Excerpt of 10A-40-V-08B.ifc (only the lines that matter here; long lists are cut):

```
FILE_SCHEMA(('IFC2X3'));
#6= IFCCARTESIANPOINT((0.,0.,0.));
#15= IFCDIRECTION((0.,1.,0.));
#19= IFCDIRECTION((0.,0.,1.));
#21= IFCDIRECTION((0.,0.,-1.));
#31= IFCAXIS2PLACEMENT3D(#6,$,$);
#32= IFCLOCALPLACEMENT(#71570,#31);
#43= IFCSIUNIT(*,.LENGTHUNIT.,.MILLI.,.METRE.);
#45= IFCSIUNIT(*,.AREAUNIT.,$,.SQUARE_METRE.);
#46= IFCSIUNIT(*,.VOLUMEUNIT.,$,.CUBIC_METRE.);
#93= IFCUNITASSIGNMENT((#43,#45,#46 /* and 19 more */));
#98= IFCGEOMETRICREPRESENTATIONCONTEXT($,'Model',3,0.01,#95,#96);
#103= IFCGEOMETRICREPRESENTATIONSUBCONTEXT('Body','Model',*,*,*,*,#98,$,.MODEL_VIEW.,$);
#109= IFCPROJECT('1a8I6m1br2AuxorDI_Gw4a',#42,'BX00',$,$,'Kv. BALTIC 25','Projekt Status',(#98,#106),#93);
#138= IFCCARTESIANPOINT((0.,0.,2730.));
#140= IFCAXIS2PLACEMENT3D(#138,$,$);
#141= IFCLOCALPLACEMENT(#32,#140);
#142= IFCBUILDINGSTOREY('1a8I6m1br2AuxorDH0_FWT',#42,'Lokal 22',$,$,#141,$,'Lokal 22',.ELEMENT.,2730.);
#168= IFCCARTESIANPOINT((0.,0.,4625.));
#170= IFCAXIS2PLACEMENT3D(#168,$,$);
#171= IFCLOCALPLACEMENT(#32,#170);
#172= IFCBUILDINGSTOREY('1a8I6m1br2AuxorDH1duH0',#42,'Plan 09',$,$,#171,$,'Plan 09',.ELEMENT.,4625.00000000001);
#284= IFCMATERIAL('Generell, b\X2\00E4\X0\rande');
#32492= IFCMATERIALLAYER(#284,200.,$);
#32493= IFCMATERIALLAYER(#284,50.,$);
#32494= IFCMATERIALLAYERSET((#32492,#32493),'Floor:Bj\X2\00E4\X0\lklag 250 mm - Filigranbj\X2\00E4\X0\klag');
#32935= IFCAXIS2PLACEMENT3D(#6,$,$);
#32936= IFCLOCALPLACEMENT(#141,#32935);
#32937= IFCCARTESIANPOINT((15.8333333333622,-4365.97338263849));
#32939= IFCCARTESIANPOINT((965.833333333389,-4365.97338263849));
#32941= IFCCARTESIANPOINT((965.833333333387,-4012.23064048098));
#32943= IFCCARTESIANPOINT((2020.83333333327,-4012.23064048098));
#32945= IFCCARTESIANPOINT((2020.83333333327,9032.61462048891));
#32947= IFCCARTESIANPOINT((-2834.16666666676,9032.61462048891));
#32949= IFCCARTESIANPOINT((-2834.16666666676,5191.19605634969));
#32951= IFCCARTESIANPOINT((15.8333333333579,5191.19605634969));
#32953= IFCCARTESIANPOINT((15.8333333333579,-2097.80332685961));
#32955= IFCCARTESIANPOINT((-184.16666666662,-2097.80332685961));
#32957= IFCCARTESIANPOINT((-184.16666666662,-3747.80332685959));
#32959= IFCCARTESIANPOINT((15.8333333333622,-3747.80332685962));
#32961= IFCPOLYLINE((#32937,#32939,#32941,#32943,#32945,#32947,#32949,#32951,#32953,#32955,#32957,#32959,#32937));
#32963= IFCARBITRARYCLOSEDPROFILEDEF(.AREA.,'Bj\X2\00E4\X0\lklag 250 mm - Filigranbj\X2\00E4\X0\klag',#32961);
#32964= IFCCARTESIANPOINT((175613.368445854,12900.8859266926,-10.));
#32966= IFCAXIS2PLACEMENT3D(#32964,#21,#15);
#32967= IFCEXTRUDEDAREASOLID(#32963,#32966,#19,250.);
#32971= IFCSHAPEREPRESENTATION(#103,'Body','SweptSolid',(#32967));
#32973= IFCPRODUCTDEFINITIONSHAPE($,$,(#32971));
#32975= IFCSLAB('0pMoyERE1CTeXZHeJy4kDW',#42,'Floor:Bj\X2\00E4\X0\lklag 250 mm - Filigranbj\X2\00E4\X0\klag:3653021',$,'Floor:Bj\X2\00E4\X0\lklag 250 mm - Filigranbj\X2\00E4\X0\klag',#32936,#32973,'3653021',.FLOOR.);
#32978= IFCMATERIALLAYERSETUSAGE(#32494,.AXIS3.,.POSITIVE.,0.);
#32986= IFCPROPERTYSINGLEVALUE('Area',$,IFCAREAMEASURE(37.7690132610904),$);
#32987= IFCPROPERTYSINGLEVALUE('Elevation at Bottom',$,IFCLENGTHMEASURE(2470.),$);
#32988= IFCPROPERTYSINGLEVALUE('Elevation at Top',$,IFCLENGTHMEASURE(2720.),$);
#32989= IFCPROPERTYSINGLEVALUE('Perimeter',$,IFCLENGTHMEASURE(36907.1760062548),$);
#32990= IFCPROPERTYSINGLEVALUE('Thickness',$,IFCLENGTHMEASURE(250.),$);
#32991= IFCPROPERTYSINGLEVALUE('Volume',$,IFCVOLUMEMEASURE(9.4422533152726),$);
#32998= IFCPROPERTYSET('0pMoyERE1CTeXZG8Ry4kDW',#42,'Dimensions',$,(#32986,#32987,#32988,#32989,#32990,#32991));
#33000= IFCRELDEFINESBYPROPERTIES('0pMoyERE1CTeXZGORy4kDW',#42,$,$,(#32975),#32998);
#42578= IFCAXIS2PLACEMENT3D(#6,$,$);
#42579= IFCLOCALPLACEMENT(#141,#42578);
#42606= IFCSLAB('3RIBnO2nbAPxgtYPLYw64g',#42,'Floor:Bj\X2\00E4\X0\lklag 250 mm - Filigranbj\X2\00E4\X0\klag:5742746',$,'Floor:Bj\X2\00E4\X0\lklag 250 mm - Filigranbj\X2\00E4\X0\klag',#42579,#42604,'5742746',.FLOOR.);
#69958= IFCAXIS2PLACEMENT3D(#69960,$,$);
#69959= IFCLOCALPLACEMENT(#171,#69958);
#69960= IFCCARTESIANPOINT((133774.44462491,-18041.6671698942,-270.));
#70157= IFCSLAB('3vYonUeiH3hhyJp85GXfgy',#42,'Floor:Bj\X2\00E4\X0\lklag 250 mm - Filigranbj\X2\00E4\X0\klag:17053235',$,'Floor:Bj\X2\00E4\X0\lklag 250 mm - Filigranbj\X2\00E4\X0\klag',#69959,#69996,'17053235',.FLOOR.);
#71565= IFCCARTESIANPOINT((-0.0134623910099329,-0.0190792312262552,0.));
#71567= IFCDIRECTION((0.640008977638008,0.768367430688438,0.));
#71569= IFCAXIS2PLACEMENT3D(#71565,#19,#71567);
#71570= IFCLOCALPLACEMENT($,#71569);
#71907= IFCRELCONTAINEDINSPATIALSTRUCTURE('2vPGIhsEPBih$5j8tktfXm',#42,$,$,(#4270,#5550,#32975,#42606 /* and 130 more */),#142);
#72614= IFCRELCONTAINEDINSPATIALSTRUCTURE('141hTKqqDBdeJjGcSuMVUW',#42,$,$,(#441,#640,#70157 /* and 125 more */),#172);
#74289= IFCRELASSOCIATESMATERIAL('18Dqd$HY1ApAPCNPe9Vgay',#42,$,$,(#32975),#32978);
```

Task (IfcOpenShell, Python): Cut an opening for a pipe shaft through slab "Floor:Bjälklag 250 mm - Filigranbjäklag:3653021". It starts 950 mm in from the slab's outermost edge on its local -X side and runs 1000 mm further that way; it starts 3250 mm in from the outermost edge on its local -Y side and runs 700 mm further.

```python
import numpy as np
import ifcopenshell
import ifcopenshell.api.feature
import ifcopenshell.api.geometry
import ifcopenshell.api.pset
import ifcopenshell.api.root
import ifcopenshell.geom
import ifcopenshell.util.element
import ifcopenshell.util.placement
import ifcopenshell.util.representation
import ifcopenshell.util.shape
import ifcopenshell.util.unit

model = ifcopenshell.open("10A-40-V-08B.ifc")
unit_scale = ifcopenshell.util.unit.calculate_unit_scale(model)
area_scale = ifcopenshell.util.unit.calculate_unit_scale(model, "AREAUNIT")
volume_scale = ifcopenshell.util.unit.calculate_unit_scale(model, "VOLUMEUNIT")
settings = ifcopenshell.geom.settings()


def volume(element):
    """Net volume in cubic metres, openings subtracted."""
    shape = ifcopenshell.geom.create_shape(settings, element)
    return ifcopenshell.util.shape.get_volume(shape.geometry)


slab = model.by_guid("0pMoyERE1CTeXZHeJy4kDW")
before = volume(slab)

# Extent in the slab's own axes, in metres. The edges named are its -X and -Y sides.
slab_shape = ifcopenshell.geom.create_shape(settings, slab)
vertices = ifcopenshell.util.shape.get_vertices(slab_shape.geometry)
x_min, y_min, bottom = vertices.min(axis=0)
top = vertices[:, 2].max()

opening = ifcopenshell.api.root.create_entity(model, ifc_class="IfcOpeningElement", name="Pipe shaft opening")
context = ifcopenshell.util.representation.get_context(model, "Model", "Body", "MODEL_VIEW")
width, depth = 1, 0.7
outline = [(0.0, 0.0), (width, 0.0), (width, depth), (0.0, depth), (0.0, 0.0)]
# Overshoot both faces by 50 mm so the cut is clean.
shape = ifcopenshell.api.geometry.add_slab_representation(
    model, context=context, depth=top - bottom + 0.1, polyline=outline
)
ifcopenshell.api.geometry.assign_representation(model, product=opening, representation=shape)

matrix = ifcopenshell.util.placement.get_local_placement(slab.ObjectPlacement)
matrix[:, 3] = matrix @ np.append(np.array([x_min + 0.95, y_min + 3.25, bottom - 0.05]) / unit_scale, 1.0)
ifcopenshell.api.geometry.edit_object_placement(model, product=opening, matrix=matrix, is_si=False)
ifcopenshell.api.feature.add_feature(model, feature=opening, element=slab)

after = volume(slab)

# Update the slab's stored quantities.
pset = model.by_id(ifcopenshell.util.element.get_pset(slab, "Dimensions", should_inherit=False)["id"])
ifcopenshell.api.pset.edit_pset(model, pset=pset, properties={
    "Area": model.create_entity("IfcAreaMeasure", after / (top - bottom) / area_scale),
    "Volume": model.create_entity("IfcVolumeMeasure", after / volume_scale),
})

print(f"slab volume {before:.3f} -> {after:.3f} m3")

model.write("10A-40-V-08B-out.ifc")
```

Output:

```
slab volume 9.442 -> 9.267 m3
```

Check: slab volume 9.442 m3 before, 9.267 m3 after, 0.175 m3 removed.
